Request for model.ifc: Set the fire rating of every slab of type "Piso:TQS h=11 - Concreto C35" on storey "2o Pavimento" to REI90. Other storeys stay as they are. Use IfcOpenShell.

First a look at what the model holds.

```python
import ifcopenshell
import ifcopenshell.util.element

model = ifcopenshell.open("model.ifc")
print(model.schema)
storey = next(s for s in model.by_type("IfcBuildingStorey") if s.Name == "2o Pavimento")
slabs = [e for e in ifcopenshell.util.element.get_decomposition(storey) if e.is_a("IfcSlab")]
seen = {}
for e in slabs:
    element_type = ifcopenshell.util.element.get_type(e)
    key = (element_type.Name if element_type != e and element_type else None, ifcopenshell.util.element.get_pset(e, "Pset_SlabCommon", "FireRating"))
    seen[key] = seen.get(key, 0) + 1
for (name, value), count in sorted(seen.items(), key=str):
    print(count, "x", name, "|", value)
```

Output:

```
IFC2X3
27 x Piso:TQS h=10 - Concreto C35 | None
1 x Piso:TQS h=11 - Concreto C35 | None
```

```python
import ifcopenshell
import ifcopenshell.api.pset
import ifcopenshell.util.element

model = ifcopenshell.open("model.ifc")

storey = next(s for s in model.by_type("IfcBuildingStorey") if s.Name == "2o Pavimento")
slabs = [e for e in ifcopenshell.util.element.get_decomposition(storey) if e.is_a("IfcSlab")]

count = 0
for e in slabs:
    element_type = ifcopenshell.util.element.get_type(e)
    if element_type in (None, e) or element_type.Name != "Piso:TQS h=11 - Concreto C35":
        continue
    # add_pset returns the element's existing set when there is one.
    pset = ifcopenshell.api.pset.add_pset(model, product=e, name="Pset_SlabCommon")
    ifcopenshell.api.pset.edit_pset(model, pset=pset, properties={"FireRating": "REI90"})
    count += 1

print(count, "slabs updated")

model.write("model-out.ifc")
```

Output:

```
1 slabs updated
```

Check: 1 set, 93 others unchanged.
